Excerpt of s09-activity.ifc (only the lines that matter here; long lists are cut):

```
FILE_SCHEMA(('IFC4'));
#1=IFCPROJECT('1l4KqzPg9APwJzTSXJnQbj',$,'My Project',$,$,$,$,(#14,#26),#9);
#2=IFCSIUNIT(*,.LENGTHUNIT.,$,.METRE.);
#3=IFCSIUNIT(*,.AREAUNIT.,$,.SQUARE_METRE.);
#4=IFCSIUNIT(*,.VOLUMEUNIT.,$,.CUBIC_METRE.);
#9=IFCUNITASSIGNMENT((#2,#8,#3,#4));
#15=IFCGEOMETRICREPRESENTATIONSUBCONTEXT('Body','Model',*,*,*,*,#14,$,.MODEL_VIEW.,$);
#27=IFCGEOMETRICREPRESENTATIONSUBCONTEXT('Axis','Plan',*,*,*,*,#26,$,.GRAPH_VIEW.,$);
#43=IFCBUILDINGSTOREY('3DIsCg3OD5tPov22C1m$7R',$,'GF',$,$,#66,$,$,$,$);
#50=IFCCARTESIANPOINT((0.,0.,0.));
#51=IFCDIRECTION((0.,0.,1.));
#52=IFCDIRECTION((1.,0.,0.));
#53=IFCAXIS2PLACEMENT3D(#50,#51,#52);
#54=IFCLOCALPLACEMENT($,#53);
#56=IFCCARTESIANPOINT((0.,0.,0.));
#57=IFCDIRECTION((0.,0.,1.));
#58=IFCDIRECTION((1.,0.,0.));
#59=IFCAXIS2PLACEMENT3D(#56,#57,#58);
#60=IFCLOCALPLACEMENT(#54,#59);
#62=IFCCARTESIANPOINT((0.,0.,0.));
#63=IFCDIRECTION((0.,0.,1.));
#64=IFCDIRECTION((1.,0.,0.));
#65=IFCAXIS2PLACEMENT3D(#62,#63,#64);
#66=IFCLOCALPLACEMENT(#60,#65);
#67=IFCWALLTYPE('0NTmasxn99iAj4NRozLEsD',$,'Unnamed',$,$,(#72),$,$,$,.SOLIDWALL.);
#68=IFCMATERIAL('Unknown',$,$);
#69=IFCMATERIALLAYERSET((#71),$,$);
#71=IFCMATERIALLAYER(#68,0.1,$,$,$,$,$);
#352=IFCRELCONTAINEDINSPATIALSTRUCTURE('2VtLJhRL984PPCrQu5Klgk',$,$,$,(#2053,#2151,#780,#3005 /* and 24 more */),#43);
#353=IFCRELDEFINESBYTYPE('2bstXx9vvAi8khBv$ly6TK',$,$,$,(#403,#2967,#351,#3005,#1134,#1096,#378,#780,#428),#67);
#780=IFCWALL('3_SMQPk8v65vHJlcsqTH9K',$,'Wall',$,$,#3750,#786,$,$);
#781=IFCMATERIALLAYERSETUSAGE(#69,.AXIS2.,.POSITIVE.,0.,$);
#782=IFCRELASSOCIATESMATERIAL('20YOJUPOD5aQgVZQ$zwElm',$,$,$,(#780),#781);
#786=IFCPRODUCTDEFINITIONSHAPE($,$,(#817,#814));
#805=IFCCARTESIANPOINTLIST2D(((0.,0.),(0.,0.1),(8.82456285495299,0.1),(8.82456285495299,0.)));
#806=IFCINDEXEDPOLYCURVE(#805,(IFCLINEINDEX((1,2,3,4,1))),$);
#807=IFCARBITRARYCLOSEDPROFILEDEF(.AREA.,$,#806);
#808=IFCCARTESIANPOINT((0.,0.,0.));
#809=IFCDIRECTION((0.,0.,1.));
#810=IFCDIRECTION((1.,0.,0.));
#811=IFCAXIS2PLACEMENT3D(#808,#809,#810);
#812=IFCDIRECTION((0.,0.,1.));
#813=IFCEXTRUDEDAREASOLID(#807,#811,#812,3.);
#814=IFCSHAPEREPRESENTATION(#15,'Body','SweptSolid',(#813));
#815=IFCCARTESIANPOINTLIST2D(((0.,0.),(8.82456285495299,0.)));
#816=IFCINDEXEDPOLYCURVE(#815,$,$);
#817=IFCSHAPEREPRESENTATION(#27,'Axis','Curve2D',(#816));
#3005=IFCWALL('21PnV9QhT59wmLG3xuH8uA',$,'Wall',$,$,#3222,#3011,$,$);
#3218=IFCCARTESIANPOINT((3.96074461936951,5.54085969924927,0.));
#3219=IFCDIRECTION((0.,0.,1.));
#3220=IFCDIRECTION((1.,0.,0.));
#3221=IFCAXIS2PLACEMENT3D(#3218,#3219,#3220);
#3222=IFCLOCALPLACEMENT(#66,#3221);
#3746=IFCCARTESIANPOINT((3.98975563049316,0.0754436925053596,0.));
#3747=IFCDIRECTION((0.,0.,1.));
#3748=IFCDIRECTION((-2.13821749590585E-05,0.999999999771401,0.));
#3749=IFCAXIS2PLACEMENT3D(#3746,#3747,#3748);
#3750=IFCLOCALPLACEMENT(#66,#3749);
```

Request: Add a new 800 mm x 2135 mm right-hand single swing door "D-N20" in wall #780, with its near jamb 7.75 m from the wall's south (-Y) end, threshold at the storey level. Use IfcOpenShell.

```python
import numpy as np
import ifcopenshell
import ifcopenshell.api.feature
import ifcopenshell.api.geometry
import ifcopenshell.api.root
import ifcopenshell.api.spatial
import ifcopenshell.geom
import ifcopenshell.util.element
import ifcopenshell.util.placement
import ifcopenshell.util.representation
import ifcopenshell.util.shape
import ifcopenshell.util.unit

model = ifcopenshell.open("s09-activity.ifc")
unit_scale = ifcopenshell.util.unit.calculate_unit_scale(model)
settings = ifcopenshell.geom.settings()


def volume(element):
    """Net volume in cubic metres, openings subtracted."""
    shape = ifcopenshell.geom.create_shape(settings, element)
    return ifcopenshell.util.shape.get_volume(shape.geometry)


wall = model.by_id(780)
storey = ifcopenshell.util.element.get_container(wall, ifc_class="IfcBuildingStorey")
context = ifcopenshell.util.representation.get_context(model, "Model", "Body", "MODEL_VIEW")
before = volume(wall)

width, height, from_end, sill = 0.8, 2.135, 7.75, 0.0  # metres

# The wall runs along its own X axis, and the end named is its -X end.
wall_shape = ifcopenshell.geom.create_shape(settings, wall)
x, y, z = ifcopenshell.util.shape.get_vertices(wall_shape.geometry).T
start = x.min() + from_end
face, thickness = float(y.min()), float(y.max() - y.min())
wall_matrix = ifcopenshell.util.placement.get_local_placement(wall.ObjectPlacement)
level = ifcopenshell.util.placement.get_local_placement(storey.ObjectPlacement)[2, 3]


def in_wall(x, y):
    """Placement at x, y metres in the wall's axes, at sill height."""
    matrix = wall_matrix.copy()
    matrix[:, 3] = wall_matrix @ np.array([x / unit_scale, y / unit_scale, 0.0, 1.0])
    matrix[2, 3] = level + sill / unit_scale
    return matrix


# Opening: a box that overshoots both wall faces by 50 mm.
opening = ifcopenshell.api.root.create_entity(model, ifc_class="IfcOpeningElement", predefined_type="OPENING")
box = ifcopenshell.api.geometry.add_wall_representation(
    model, context=context, length=width, height=height, thickness=thickness + 0.1
)
ifcopenshell.api.geometry.assign_representation(model, product=opening, representation=box)
ifcopenshell.api.geometry.edit_object_placement(model, product=opening, matrix=in_wall(start, face - 0.05), is_si=False)
ifcopenshell.api.feature.add_feature(model, feature=opening, element=wall)

door = ifcopenshell.api.root.create_entity(model, ifc_class="IfcDoor", name="D-N20", predefined_type="DOOR")
door.OverallWidth, door.OverallHeight = width / unit_scale, height / unit_scale
door.OperationType = "SINGLE_SWING_RIGHT"
body = ifcopenshell.api.geometry.add_door_representation(
    model,
    context=context,
    overall_width=door.OverallWidth,
    overall_height=door.OverallHeight,
    operation_type="SINGLE_SWING_RIGHT",
    lining_properties={"LiningDepth": thickness / unit_scale, "ThresholdDepth": thickness / unit_scale},
)
ifcopenshell.api.geometry.assign_representation(model, product=door, representation=body)
ifcopenshell.api.spatial.assign_container(model, products=[door], relating_structure=storey)
ifcopenshell.api.feature.add_filling(model, opening=opening, element=door)

# The lining spans the wall, so the door starts at the wall face.
ifcopenshell.api.geometry.edit_object_placement(model, product=door, matrix=in_wall(start, face), is_si=False)

after = volume(wall)

print(f"wall volume {before:.3f} -> {after:.3f} m3")

model.write("s09-activity_v2.ifc")
```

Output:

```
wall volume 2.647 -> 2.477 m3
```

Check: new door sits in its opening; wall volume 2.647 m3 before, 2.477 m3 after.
